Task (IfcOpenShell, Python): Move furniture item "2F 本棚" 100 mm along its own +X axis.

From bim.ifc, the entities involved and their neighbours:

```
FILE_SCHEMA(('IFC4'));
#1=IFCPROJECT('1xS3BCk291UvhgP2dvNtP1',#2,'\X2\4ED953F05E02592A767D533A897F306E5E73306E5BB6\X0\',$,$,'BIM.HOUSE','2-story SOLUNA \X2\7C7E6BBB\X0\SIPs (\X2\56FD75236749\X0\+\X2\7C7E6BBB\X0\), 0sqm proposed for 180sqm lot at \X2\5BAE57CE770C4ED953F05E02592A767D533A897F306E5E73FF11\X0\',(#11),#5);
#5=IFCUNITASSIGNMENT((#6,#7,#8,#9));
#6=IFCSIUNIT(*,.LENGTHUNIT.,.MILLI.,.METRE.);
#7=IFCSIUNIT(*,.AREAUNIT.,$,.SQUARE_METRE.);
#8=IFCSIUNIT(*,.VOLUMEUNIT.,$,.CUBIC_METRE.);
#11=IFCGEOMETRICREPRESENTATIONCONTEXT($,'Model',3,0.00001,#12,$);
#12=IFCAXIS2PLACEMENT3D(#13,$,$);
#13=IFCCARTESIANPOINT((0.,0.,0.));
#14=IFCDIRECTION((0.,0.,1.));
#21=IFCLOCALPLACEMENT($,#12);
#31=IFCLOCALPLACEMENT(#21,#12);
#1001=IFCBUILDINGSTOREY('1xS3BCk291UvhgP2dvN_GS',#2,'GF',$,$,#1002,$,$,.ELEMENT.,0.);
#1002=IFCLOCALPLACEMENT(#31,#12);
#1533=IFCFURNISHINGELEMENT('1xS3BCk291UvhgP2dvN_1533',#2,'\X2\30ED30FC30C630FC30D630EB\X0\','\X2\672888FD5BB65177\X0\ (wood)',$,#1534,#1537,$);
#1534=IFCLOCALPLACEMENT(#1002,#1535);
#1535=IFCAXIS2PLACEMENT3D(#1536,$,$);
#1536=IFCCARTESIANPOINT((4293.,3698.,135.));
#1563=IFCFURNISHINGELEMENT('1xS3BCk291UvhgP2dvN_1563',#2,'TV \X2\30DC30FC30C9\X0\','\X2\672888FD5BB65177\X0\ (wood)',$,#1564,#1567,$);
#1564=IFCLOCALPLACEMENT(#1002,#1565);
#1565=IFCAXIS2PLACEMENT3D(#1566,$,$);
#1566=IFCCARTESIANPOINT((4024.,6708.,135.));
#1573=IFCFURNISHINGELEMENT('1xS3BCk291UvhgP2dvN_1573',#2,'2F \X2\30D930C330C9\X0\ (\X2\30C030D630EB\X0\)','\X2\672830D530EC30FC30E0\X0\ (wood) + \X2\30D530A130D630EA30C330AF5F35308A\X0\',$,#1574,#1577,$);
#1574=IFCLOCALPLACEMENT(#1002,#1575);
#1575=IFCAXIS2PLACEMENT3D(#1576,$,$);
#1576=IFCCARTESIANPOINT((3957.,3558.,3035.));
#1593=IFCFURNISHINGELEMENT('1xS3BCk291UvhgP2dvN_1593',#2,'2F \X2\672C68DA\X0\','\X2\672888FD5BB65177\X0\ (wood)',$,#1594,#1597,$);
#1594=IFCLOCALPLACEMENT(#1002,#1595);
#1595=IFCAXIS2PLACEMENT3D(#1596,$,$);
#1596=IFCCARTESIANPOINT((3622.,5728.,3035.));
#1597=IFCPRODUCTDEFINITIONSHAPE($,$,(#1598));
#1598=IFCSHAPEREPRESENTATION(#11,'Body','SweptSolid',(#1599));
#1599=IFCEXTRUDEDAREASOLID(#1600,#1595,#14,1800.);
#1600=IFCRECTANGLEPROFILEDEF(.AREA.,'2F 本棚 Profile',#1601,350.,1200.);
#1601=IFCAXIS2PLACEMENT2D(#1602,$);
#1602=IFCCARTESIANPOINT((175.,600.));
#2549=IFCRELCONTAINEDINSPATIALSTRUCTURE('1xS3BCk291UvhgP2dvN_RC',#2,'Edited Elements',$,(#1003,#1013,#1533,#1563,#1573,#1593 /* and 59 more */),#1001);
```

```python
import ifcopenshell
import ifcopenshell.api.geometry
import ifcopenshell.util.placement
import ifcopenshell.util.unit

model = ifcopenshell.open("bim.ifc")
unit_scale = ifcopenshell.util.unit.calculate_unit_scale(model)

item = model.by_guid("1xS3BCk291UvhgP2dvN_1593")
matrix = ifcopenshell.util.placement.get_local_placement(item.ObjectPlacement)
matrix[:3, 3] += matrix[:3, 0] * 0.1 / unit_scale
ifcopenshell.api.geometry.edit_object_placement(model, product=item, matrix=matrix, is_si=False)

print(ifcopenshell.util.placement.get_local_placement(item.ObjectPlacement).round(3) + 0.0)

model.write("bim_rev.ifc")
```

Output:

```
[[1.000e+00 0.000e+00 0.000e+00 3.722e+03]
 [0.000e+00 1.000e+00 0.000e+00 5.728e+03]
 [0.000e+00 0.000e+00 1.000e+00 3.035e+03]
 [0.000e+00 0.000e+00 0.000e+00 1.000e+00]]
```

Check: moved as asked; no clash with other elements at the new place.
